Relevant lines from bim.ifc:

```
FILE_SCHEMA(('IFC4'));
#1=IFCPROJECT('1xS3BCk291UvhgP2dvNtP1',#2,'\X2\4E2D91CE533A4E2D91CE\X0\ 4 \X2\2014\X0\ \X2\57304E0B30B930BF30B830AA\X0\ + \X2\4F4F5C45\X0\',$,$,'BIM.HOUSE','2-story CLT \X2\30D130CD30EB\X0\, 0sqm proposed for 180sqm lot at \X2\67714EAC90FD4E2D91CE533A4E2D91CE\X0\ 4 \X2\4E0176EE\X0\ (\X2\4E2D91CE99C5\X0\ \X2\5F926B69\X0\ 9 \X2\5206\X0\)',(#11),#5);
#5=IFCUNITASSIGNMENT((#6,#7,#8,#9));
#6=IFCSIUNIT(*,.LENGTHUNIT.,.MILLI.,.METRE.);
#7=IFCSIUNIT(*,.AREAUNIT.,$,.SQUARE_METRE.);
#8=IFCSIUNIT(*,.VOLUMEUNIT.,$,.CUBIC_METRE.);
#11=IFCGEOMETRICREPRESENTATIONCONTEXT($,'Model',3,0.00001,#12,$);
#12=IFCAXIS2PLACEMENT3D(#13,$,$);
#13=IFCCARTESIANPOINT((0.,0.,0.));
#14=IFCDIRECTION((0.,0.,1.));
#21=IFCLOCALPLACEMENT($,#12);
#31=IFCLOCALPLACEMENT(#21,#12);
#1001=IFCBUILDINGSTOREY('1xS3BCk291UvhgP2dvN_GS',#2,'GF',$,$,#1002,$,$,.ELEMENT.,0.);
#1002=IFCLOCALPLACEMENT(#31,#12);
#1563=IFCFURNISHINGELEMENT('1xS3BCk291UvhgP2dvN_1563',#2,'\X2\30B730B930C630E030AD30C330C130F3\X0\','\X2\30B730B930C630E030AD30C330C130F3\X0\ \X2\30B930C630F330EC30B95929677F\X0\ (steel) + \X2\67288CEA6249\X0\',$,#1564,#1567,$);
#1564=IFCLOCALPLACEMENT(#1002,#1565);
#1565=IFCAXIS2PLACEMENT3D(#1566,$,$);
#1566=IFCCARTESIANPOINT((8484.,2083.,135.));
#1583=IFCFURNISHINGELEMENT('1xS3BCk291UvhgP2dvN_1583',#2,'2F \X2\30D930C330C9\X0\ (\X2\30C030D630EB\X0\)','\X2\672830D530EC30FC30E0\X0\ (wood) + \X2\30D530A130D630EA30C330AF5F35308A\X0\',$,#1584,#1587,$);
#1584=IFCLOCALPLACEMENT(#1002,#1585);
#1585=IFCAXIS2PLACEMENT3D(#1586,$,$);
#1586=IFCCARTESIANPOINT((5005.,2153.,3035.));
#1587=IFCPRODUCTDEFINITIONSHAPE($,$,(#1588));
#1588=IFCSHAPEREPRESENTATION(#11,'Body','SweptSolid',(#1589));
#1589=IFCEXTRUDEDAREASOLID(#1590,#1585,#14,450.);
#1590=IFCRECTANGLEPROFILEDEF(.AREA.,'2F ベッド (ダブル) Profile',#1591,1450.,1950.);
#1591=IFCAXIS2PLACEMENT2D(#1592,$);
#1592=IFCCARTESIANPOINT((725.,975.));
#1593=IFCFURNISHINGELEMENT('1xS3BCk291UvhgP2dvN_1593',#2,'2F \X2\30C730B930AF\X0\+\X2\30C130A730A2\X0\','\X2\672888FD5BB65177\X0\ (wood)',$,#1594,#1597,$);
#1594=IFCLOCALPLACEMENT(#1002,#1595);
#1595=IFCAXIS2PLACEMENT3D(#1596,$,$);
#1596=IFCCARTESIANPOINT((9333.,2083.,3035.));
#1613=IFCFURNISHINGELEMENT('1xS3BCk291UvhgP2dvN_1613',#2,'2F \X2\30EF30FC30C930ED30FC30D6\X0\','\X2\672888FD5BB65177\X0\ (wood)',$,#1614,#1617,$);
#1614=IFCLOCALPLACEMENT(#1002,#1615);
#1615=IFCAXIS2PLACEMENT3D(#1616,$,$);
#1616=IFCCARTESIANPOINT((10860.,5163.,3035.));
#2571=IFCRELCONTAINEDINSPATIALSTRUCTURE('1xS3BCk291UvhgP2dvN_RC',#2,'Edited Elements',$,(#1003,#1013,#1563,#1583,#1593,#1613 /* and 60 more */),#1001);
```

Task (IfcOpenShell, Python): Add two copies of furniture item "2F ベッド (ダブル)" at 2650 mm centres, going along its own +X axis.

```python
import ifcopenshell
import ifcopenshell.api.geometry
import ifcopenshell.api.root
import ifcopenshell.util.element
import ifcopenshell.util.placement
import ifcopenshell.util.unit

model = ifcopenshell.open("bim.ifc")
unit_scale = ifcopenshell.util.unit.calculate_unit_scale(model)


def reuse_history(source, copy):
    """copy_class also copies each property set's owner history, people and application; keep the originals."""
    for rel in copy.IsDefinedBy:
        if rel.is_a("IfcRelDefinesByProperties") and (history := rel.RelatingPropertyDefinition.OwnerHistory):
            rel.RelatingPropertyDefinition.OwnerHistory = source.OwnerHistory
            ifcopenshell.util.element.remove_deep2(model, history)


source = model.by_id(1583)
base = ifcopenshell.util.placement.get_local_placement(source.ObjectPlacement)
step = base[:3, 0] * 2.65 / unit_scale

for i in range(1, 3):
    copy = ifcopenshell.api.root.copy_class(model, product=source)
    copy.Representation = ifcopenshell.util.element.copy_deep(
        model, source.Representation, exclude=["IfcGeometricRepresentationContext", "IfcRepresentationMap"]
    )
    reuse_history(source, copy)
    matrix = base.copy()
    matrix[:3, 3] += i * step
    print("added at", matrix[:3, 3].round(3) + 0.0)
    ifcopenshell.api.geometry.edit_object_placement(model, product=copy, matrix=matrix, is_si=False)

model.write("bim-out.ifc")
```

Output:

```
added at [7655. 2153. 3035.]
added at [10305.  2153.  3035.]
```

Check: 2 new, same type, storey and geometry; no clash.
